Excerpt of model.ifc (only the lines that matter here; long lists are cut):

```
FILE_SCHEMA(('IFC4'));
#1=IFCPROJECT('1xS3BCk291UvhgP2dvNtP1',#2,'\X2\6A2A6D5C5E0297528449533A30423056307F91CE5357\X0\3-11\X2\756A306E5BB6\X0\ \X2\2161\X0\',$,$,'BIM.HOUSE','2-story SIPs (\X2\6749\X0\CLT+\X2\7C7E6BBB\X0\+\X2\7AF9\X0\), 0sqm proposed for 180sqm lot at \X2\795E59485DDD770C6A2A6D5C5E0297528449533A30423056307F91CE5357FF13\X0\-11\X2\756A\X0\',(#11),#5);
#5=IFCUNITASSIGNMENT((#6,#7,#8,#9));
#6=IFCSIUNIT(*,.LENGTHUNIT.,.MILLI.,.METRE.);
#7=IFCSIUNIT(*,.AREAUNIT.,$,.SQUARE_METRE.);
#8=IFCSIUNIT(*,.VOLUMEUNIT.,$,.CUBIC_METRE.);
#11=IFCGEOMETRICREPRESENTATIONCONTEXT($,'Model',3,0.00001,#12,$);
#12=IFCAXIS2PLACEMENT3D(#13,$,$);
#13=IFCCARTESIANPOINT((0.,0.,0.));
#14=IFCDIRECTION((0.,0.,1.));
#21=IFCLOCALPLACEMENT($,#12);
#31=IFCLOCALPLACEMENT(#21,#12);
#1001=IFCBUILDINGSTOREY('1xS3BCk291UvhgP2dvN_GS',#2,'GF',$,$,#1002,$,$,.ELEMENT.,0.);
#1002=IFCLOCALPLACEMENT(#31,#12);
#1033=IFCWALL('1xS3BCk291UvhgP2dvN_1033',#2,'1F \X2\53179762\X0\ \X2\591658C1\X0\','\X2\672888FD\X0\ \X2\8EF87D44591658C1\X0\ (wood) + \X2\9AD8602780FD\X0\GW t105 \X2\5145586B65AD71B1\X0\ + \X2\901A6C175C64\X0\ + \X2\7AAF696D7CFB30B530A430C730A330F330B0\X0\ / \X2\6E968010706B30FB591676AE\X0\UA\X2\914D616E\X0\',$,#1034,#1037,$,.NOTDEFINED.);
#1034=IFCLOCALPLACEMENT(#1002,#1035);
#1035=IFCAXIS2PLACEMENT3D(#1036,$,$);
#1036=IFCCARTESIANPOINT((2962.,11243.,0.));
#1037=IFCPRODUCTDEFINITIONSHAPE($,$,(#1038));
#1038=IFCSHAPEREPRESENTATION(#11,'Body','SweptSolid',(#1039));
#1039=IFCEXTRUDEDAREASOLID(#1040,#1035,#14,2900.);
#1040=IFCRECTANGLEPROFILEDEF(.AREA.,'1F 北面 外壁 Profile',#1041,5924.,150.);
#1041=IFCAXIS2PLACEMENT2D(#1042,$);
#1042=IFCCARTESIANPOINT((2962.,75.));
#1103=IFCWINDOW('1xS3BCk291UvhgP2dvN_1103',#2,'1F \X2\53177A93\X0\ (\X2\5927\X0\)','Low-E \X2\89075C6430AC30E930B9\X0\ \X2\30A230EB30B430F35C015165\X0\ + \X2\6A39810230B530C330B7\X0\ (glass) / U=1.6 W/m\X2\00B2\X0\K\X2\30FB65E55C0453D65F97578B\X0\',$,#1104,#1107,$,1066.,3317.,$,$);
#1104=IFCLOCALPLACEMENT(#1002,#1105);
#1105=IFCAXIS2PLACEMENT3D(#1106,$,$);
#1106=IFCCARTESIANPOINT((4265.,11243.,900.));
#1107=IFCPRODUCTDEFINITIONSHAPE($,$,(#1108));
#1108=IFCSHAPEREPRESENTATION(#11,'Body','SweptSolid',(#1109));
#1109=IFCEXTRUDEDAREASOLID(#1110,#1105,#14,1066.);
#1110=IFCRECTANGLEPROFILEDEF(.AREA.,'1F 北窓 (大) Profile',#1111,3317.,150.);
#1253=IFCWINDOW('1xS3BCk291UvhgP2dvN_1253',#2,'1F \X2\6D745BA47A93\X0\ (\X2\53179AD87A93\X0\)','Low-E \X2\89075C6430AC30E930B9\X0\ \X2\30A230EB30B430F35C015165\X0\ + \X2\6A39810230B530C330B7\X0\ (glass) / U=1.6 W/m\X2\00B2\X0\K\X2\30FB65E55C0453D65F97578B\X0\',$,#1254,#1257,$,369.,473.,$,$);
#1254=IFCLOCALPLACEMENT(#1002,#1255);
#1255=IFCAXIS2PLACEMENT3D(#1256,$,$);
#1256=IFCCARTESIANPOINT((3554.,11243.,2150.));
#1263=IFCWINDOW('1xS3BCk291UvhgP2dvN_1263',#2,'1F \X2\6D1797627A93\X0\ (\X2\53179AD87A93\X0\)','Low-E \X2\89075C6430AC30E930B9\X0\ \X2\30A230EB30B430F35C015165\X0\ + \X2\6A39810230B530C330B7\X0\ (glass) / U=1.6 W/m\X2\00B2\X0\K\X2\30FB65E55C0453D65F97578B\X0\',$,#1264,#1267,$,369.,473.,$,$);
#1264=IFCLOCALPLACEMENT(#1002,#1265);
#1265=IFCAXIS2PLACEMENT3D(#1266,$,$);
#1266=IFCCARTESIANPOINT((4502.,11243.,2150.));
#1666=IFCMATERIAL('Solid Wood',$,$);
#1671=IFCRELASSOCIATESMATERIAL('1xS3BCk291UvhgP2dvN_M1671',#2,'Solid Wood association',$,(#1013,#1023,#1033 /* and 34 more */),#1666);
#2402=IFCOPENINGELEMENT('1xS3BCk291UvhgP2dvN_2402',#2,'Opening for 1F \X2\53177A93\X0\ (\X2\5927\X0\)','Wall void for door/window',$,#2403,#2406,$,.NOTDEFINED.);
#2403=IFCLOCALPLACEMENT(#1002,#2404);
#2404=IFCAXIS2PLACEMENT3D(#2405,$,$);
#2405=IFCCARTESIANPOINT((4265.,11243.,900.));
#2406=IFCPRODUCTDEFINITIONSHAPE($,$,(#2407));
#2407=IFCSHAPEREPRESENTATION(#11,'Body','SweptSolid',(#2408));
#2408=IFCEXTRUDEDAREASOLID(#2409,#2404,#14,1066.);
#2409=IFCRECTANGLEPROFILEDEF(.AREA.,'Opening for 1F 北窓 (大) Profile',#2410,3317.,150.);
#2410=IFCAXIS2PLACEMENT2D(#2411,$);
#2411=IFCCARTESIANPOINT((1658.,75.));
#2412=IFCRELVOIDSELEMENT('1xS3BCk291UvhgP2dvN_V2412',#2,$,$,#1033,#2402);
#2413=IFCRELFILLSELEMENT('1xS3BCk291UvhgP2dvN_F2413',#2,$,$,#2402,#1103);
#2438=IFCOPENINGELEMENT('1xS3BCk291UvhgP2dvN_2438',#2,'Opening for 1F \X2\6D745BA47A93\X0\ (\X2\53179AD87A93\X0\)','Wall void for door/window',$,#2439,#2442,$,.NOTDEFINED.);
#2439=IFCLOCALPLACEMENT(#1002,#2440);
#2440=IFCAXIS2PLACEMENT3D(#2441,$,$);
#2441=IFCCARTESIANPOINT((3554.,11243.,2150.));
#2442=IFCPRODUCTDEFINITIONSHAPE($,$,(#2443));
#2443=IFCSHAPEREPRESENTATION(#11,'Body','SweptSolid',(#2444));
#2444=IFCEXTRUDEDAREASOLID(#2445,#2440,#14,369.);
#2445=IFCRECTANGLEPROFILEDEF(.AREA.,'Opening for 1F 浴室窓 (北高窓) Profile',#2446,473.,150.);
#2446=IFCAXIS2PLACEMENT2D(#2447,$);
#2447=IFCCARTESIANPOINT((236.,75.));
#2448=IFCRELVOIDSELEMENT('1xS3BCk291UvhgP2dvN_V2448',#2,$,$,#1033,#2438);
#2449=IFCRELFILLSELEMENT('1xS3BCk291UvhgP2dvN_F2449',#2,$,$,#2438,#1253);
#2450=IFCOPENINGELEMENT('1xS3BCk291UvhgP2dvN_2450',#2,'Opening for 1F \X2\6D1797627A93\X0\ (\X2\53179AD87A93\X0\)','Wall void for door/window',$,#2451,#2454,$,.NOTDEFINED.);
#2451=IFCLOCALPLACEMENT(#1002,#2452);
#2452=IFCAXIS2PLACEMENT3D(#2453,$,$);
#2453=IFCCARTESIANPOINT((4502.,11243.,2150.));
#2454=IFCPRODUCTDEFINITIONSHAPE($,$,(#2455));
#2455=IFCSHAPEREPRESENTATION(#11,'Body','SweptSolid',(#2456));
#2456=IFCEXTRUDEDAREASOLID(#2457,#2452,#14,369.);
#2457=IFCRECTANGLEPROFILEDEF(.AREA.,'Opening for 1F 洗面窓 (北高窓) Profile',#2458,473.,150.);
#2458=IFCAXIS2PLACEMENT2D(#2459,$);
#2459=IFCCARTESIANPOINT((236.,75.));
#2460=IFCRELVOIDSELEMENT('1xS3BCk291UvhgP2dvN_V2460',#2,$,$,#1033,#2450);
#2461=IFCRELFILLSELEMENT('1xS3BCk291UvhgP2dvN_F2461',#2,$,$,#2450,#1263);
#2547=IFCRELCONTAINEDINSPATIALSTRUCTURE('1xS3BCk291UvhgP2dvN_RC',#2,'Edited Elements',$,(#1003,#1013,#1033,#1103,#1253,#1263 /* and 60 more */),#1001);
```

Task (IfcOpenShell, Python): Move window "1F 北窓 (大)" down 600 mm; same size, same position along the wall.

```python
import numpy as np
import ifcopenshell
import ifcopenshell.api.geometry
import ifcopenshell.util.placement
import ifcopenshell.util.unit

model = ifcopenshell.open("model.ifc")
unit_scale = ifcopenshell.util.unit.calculate_unit_scale(model)

window = model.by_guid("1xS3BCk291UvhgP2dvN_1103")
opening = window.FillsVoids[0].RelatingOpeningElement
dz = -0.6 / unit_scale

shift = np.array([0.0, 0.0, dz])
# The window is not placed relative to its opening, so move both.
for product in (opening, window):
    matrix = ifcopenshell.util.placement.get_local_placement(product.ObjectPlacement)
    matrix[:3, 3] += shift
    ifcopenshell.api.geometry.edit_object_placement(model, product=product, matrix=matrix, is_si=False)

print(f"moved by {dz * unit_scale:+.3f} m")

model.write("model_edited.ifc")
```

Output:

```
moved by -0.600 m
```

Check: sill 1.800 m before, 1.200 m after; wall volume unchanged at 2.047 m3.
